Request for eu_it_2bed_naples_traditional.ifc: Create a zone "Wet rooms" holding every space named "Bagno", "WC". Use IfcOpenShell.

First a look at what the model holds.

```python
import ifcopenshell

model = ifcopenshell.open("eu_it_2bed_naples_traditional.ifc")
print(model.schema)
seen = {}
for space in model.by_type("IfcSpace"):
    seen[space.LongName] = seen.get(space.LongName, 0) + 1
for name, count in sorted(seen.items(), key=str):
    print(count, "x", name)
print("zones:", [z.Name for z in model.by_type("IfcZone")][:20])
```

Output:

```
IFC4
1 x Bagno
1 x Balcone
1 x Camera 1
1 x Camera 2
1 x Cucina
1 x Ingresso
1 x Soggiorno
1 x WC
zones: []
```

```python
import ifcopenshell
import ifcopenshell.api.group
import ifcopenshell.api.root

model = ifcopenshell.open("eu_it_2bed_naples_traditional.ifc")

names = {"Bagno", "WC"}
spaces = [s for s in model.by_type("IfcSpace") if s.LongName in names]

zone = ifcopenshell.api.root.create_entity(model, ifc_class="IfcZone", name="Wet rooms")
ifcopenshell.api.group.assign_group(model, products=spaces, group=zone)
print(len(spaces), "spaces in", zone.Name)

model.write("eu_it_2bed_naples_traditional_v2.ifc")
```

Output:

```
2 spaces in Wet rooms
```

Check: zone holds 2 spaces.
